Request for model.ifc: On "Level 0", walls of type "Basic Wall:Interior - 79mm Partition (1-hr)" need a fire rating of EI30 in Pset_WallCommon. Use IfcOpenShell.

First a look at what the model holds.

```python
import ifcopenshell
import ifcopenshell.util.element

model = ifcopenshell.open("model.ifc")
print(model.schema)
storey = next(s for s in model.by_type("IfcBuildingStorey") if s.Name == "Level 0")
walls = [e for e in ifcopenshell.util.element.get_decomposition(storey) if e.is_a("IfcWall")]
seen = {}
for e in walls:
    element_type = ifcopenshell.util.element.get_type(e)
    key = (element_type.Name if element_type != e and element_type else None, ifcopenshell.util.element.get_pset(e, "Pset_WallCommon", "FireRating"))
    seen[key] = seen.get(key, 0) + 1
for (name, value), count in sorted(seen.items(), key=str):
    print(count, "x", name, "|", value)
```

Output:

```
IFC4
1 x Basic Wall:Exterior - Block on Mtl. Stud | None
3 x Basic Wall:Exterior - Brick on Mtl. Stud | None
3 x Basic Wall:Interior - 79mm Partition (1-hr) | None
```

```python
import ifcopenshell
import ifcopenshell.api.pset
import ifcopenshell.util.element

model = ifcopenshell.open("model.ifc")

storey = next(s for s in model.by_type("IfcBuildingStorey") if s.Name == "Level 0")
walls = [e for e in ifcopenshell.util.element.get_decomposition(storey) if e.is_a("IfcWall")]

count = 0
for e in walls:
    element_type = ifcopenshell.util.element.get_type(e)
    if element_type in (None, e) or element_type.Name != "Basic Wall:Interior - 79mm Partition (1-hr)":
        continue
    # add_pset returns the element's existing set when there is one.
    pset = ifcopenshell.api.pset.add_pset(model, product=e, name="Pset_WallCommon")
    ifcopenshell.api.pset.edit_pset(model, pset=pset, properties={"FireRating": "EI30"})
    count += 1

print(count, "walls updated")

model.write("model_updated.ifc")
```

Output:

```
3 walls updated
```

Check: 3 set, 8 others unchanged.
